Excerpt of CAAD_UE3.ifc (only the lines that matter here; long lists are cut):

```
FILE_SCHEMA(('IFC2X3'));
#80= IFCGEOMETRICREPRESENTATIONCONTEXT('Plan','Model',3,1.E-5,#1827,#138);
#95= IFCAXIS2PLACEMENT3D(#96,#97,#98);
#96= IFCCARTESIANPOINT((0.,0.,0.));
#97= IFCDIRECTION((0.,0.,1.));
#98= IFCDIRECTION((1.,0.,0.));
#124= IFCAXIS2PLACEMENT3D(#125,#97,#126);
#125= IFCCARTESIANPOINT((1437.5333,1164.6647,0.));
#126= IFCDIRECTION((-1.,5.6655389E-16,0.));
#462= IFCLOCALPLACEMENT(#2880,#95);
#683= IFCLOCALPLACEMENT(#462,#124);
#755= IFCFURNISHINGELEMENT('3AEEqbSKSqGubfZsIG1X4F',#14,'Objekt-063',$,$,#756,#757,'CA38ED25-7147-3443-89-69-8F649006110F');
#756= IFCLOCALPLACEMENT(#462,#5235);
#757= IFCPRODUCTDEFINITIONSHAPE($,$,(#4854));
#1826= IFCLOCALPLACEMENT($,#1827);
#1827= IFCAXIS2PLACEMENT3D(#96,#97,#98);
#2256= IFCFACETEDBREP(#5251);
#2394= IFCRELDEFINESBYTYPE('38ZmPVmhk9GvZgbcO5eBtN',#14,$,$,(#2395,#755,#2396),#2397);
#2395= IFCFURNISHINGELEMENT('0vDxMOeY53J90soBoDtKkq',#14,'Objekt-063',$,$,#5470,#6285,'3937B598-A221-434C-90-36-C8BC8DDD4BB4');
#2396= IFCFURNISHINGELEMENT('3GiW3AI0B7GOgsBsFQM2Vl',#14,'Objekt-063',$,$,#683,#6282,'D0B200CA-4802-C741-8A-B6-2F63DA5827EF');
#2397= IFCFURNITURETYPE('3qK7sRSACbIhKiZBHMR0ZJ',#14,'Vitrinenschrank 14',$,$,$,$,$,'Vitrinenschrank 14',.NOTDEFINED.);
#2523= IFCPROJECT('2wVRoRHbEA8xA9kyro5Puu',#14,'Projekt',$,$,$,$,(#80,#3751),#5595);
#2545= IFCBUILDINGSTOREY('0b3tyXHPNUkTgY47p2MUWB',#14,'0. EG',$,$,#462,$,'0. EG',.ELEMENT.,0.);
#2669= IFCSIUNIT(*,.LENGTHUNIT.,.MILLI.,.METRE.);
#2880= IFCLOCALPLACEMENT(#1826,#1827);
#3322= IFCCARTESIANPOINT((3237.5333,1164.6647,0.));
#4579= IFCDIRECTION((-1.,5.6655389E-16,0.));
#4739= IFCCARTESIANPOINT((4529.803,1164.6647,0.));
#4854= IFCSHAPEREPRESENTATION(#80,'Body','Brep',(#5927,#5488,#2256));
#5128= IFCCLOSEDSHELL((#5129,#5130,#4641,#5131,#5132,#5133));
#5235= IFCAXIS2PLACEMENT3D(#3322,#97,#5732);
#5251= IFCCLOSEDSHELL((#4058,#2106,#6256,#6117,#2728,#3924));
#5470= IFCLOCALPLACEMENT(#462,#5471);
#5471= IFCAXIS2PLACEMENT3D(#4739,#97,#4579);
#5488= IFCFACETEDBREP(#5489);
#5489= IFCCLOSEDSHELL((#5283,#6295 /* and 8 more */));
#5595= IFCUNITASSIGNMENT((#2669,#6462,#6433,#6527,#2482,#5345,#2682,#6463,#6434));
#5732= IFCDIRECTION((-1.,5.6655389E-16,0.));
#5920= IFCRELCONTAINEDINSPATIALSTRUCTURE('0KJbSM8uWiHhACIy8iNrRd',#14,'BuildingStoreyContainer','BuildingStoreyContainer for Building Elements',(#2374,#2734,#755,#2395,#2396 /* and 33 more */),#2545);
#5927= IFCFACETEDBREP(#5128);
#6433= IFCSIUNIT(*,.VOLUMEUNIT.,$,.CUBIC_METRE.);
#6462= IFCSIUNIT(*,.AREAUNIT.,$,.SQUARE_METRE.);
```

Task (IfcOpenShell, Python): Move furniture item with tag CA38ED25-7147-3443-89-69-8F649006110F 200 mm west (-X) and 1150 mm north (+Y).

```python
import ifcopenshell
import ifcopenshell.api.geometry
import ifcopenshell.util.placement
import ifcopenshell.util.unit

model = ifcopenshell.open("CAAD_UE3.ifc")
unit_scale = ifcopenshell.util.unit.calculate_unit_scale(model)

item = model.by_guid("3AEEqbSKSqGubfZsIG1X4F")
matrix = ifcopenshell.util.placement.get_local_placement(item.ObjectPlacement)
matrix[0, 3] -= 0.2 / unit_scale
matrix[1, 3] += 1.15 / unit_scale
ifcopenshell.api.geometry.edit_object_placement(model, product=item, matrix=matrix, is_si=False)

print(ifcopenshell.util.placement.get_local_placement(item.ObjectPlacement).round(3) + 0.0)

model.write("CAAD_UE3_rev.ifc")
```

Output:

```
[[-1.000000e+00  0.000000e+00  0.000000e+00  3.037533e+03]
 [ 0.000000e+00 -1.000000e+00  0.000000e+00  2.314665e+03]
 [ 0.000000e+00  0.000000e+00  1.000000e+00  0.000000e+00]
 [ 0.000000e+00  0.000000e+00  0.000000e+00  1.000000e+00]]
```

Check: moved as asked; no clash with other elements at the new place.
